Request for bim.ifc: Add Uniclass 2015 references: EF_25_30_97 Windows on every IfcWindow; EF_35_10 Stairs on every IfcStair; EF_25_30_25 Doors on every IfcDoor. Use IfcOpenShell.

First a look at what the model holds.

```python
import ifcopenshell

model = ifcopenshell.open("bim.ifc")
print(model.schema)
print("classifications:", [c.Name for c in model.by_type("IfcClassification")])
for ifc_class in ("IfcDoor", "IfcRoof", "IfcStair", "IfcWall", "IfcWindow"):
    print(ifc_class, len(model.by_type(ifc_class)))
```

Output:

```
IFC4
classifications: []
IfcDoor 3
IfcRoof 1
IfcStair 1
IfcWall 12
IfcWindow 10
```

```python
import ifcopenshell
import ifcopenshell.api.classification

model = ifcopenshell.open("bim.ifc")

system = ifcopenshell.api.classification.add_classification(model, classification="Uniclass 2015")

codes = {
    "IfcWindow": ("EF_25_30_97", "Windows"),
    "IfcStair": ("EF_35_10", "Stairs"),
    "IfcDoor": ("EF_25_30_25", "Doors"),
}
for ifc_class, (code, name) in codes.items():
    products = model.by_type(ifc_class)
    ifcopenshell.api.classification.add_reference(
        model, products=products, classification=system, identification=code, name=name
    )
    print(code, len(products))

model.write("bim_rev.ifc")
```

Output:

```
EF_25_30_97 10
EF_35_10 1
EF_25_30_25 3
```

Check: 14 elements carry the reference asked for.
